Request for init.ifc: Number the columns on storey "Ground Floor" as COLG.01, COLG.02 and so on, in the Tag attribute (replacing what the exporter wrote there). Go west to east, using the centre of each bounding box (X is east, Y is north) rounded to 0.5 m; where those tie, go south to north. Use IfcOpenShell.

First a look at what the model holds.

```python
import ifcopenshell
import ifcopenshell.util.element
import ifcopenshell.util.placement

model = ifcopenshell.open("init.ifc")
print(model.schema)
storey = next(s for s in model.by_type("IfcBuildingStorey") if s.Name == "Ground Floor")
columns = [e for e in ifcopenshell.util.element.get_decomposition(storey) if e.is_a("IfcColumn")]
for e in sorted(columns, key=lambda e: e.id()):
    origin = ifcopenshell.util.placement.get_local_placement(e.ObjectPlacement)[:3, 3]
    print(e.id(), e.Tag, e.Name, origin.round(2) + 0.0, sep=" | ")
```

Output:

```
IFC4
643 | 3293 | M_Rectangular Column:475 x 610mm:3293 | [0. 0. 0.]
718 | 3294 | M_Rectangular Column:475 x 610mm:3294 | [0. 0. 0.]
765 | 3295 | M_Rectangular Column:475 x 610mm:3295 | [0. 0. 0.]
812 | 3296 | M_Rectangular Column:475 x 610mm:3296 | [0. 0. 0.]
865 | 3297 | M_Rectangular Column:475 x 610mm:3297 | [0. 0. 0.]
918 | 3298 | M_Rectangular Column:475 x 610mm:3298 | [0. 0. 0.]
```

```python
import ifcopenshell
import ifcopenshell.geom
import ifcopenshell.util.element
import ifcopenshell.util.shape

model = ifcopenshell.open("init.ifc")
settings = ifcopenshell.geom.settings()
settings.set("use-world-coords", True)


def centre(element):
    shape = ifcopenshell.geom.create_shape(settings, element)
    return ifcopenshell.util.shape.get_bbox_centroid(shape.geometry)


storey = next(s for s in model.by_type("IfcBuildingStorey") if s.Name == "Ground Floor")
columns = [e for e in ifcopenshell.util.element.get_decomposition(storey) if e.is_a("IfcColumn")]

# Insertion points can sit at a corner or the storey origin, so sort by the geometry (in metres).
centres = {e: centre(e) for e in columns}
columns.sort(key=lambda e: (round(centres[e][0] / 0.5), centres[e][1]))

for i, e in enumerate(columns, start=1):
    number = f"COLG.{i:02d}"
    e.Tag = number
    print(e.id(), number)

model.write("init_v2.ifc")
```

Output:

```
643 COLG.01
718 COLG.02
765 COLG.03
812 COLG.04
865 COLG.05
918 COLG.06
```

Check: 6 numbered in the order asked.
